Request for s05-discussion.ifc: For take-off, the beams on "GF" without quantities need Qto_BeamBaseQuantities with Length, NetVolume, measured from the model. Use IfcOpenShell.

First a look at what the model holds.

```python
import ifcopenshell
import ifcopenshell.util.element
import ifcopenshell.util.unit

model = ifcopenshell.open("s05-discussion.ifc")
print(model.schema)
for unit_type in ("LENGTHUNIT", "AREAUNIT", "VOLUMEUNIT"):
    print(unit_type, ifcopenshell.util.unit.calculate_unit_scale(model, unit_type))
storey = next(s for s in model.by_type("IfcBuildingStorey") if s.Name == "GF")
beams = [e for e in ifcopenshell.util.element.get_decomposition(storey) if e.is_a("IfcBeam")]
for e in sorted(beams, key=lambda e: e.id()):
    print(e.id(), e.is_a(), e.Name, list(ifcopenshell.util.element.get_psets(e, qtos_only=True)), sep=" | ")
```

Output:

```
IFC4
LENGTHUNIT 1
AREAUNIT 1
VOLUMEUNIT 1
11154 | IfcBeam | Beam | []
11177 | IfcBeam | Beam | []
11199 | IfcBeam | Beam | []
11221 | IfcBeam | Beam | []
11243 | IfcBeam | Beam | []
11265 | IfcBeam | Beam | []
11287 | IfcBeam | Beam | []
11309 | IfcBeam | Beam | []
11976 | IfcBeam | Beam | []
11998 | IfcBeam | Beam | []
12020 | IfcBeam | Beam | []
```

```python
import ifcopenshell
import ifcopenshell.api.pset
import ifcopenshell.geom
import ifcopenshell.util.element
import ifcopenshell.util.shape
import ifcopenshell.util.unit

model = ifcopenshell.open("s05-discussion.ifc")
unit_scale = ifcopenshell.util.unit.calculate_unit_scale(model)
volume_scale = ifcopenshell.util.unit.calculate_unit_scale(model, "VOLUMEUNIT")
settings = ifcopenshell.geom.settings()

storey = next(s for s in model.by_type("IfcBuildingStorey") if s.Name == "GF")
beams = [e for e in ifcopenshell.util.element.get_decomposition(storey) if e.is_a("IfcBeam")]

for e in sorted(beams, key=lambda e: e.id()):
    if ifcopenshell.util.element.get_psets(e, qtos_only=True, should_inherit=False):
        continue
    # Geometry comes back in metres, in the element's own axes.
    shape = ifcopenshell.geom.create_shape(settings, e)
    values = {
        "Length": ifcopenshell.util.shape.get_max_xyz(shape.geometry) / unit_scale,
        "NetVolume": ifcopenshell.util.shape.get_volume(shape.geometry) / volume_scale,
    }
    qto = ifcopenshell.api.pset.add_qto(model, product=e, name="Qto_BeamBaseQuantities")
    ifcopenshell.api.pset.edit_qto(model, qto=qto, properties=values)
    print(e.id(), {k: round(v, 3) for k, v in values.items()})

model.write("s05-discussion_edited.ifc")
```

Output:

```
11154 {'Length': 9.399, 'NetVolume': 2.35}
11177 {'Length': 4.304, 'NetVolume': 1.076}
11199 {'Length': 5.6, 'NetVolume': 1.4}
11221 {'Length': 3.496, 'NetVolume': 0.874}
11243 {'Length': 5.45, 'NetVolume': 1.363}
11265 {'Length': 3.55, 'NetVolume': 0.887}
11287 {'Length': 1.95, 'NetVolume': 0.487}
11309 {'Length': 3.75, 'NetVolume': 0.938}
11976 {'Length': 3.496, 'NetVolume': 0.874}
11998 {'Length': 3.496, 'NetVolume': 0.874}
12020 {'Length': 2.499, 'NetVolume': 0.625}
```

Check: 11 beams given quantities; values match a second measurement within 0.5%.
